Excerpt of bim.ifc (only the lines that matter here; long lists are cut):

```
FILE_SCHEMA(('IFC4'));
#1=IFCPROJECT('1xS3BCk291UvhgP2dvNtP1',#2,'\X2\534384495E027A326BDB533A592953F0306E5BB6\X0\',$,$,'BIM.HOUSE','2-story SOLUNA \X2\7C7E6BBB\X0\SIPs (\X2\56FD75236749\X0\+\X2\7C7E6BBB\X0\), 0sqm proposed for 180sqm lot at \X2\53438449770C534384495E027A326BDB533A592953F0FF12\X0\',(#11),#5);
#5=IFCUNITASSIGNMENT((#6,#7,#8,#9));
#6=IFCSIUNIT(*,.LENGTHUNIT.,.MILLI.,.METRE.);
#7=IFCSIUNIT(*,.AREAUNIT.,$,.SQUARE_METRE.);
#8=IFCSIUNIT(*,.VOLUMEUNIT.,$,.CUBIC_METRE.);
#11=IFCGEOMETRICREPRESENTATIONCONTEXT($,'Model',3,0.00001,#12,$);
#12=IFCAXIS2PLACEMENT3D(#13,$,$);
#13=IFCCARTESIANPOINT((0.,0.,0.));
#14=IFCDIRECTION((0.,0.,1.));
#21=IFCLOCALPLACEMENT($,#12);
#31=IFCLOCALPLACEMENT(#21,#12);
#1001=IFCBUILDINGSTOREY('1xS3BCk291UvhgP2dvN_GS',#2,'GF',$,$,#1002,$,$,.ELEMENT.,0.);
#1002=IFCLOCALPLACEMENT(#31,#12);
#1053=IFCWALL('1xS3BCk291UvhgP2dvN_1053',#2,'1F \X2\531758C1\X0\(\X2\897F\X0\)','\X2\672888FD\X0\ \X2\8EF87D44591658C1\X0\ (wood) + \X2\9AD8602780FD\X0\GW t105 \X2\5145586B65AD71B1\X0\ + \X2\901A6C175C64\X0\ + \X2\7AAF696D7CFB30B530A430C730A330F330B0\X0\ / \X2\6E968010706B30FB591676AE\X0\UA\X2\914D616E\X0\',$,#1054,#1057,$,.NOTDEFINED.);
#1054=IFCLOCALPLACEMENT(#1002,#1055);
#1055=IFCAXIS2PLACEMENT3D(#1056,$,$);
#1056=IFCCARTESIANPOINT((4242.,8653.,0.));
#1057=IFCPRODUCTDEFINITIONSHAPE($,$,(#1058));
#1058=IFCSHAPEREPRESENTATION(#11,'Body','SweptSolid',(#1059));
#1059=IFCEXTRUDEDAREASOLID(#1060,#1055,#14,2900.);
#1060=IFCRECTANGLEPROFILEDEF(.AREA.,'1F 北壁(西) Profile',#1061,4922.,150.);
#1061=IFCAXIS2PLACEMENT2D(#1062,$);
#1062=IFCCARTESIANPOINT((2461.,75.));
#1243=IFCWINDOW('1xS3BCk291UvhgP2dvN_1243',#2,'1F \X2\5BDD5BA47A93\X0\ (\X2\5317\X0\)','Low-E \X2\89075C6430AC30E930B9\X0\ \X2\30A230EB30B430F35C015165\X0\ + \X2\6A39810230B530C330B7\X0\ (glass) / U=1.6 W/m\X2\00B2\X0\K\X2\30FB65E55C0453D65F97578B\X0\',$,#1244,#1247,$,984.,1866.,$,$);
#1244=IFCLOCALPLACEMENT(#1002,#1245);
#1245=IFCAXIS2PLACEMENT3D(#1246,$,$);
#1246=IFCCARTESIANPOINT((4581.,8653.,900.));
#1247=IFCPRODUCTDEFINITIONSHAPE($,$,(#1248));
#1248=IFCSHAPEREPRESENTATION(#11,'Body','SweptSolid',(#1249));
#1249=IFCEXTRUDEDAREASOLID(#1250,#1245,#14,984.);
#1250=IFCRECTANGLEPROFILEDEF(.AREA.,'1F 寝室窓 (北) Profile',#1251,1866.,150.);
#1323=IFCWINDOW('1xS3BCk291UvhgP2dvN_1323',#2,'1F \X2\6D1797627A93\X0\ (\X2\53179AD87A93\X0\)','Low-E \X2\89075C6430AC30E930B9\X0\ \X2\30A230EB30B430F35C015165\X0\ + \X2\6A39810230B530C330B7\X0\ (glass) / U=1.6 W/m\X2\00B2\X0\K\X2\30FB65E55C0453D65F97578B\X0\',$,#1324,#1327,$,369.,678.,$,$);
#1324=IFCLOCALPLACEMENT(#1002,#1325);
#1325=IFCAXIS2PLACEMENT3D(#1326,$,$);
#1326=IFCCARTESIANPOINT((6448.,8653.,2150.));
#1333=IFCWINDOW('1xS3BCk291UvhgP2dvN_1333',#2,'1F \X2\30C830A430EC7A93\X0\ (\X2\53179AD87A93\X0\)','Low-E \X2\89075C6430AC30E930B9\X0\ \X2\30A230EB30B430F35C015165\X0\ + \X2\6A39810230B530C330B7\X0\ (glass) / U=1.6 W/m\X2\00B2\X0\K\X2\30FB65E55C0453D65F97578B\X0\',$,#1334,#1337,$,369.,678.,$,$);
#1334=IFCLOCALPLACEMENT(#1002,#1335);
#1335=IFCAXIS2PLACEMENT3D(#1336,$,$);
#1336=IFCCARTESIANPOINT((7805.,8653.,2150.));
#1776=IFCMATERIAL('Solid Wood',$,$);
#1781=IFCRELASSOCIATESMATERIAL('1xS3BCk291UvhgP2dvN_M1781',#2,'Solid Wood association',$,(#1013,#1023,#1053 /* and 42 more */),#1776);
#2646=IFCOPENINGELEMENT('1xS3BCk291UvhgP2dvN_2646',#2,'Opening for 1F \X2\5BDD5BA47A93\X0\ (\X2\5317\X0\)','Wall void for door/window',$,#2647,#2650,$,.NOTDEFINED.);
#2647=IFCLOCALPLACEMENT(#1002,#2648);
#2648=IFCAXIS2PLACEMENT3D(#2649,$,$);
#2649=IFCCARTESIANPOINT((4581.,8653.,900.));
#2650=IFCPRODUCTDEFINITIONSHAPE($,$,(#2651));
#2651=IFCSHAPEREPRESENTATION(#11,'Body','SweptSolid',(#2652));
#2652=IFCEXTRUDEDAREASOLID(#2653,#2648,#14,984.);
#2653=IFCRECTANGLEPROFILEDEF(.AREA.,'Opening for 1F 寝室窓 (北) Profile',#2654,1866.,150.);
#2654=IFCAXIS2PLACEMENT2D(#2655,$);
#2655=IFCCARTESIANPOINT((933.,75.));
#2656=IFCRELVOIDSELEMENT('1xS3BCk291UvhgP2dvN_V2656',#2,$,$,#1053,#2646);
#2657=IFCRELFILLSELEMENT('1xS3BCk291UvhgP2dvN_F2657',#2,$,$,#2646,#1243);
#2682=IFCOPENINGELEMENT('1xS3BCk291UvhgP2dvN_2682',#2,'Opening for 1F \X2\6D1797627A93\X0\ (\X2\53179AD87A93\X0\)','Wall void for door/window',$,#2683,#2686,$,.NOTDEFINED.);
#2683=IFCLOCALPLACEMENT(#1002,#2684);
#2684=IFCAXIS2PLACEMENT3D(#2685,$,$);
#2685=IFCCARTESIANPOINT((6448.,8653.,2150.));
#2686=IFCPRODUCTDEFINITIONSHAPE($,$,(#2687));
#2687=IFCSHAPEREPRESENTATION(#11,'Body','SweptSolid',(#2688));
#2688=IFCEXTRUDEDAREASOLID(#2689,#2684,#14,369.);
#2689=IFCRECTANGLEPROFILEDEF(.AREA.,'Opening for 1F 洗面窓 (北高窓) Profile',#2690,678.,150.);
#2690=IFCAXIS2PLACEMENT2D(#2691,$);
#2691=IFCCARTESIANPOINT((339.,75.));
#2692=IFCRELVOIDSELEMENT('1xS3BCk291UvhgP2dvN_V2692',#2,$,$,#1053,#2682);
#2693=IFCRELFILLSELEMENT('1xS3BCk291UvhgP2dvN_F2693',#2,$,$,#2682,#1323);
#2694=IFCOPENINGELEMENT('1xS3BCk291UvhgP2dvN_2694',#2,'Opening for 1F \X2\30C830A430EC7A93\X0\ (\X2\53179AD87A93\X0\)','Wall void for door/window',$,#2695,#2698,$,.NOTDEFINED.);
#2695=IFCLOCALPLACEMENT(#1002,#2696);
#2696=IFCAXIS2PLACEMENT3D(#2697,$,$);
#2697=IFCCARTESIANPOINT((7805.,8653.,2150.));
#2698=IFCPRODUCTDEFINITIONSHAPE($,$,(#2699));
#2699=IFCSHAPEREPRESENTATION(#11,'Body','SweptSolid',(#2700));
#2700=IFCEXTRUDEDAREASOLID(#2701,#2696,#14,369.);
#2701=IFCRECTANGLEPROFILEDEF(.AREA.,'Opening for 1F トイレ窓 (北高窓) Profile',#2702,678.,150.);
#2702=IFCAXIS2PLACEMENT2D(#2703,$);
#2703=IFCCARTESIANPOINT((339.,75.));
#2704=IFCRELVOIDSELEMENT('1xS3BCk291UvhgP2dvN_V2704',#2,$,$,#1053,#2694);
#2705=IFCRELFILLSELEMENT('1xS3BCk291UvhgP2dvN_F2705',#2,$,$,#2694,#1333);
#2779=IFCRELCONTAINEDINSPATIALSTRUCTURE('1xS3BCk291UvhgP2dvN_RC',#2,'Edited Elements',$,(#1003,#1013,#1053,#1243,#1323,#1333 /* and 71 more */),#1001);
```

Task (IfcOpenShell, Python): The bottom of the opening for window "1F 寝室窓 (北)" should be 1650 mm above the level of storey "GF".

```python
import numpy as np
import ifcopenshell
import ifcopenshell.api.geometry
import ifcopenshell.geom
import ifcopenshell.util.element
import ifcopenshell.util.placement
import ifcopenshell.util.shape
import ifcopenshell.util.unit

model = ifcopenshell.open("bim.ifc")
unit_scale = ifcopenshell.util.unit.calculate_unit_scale(model)

window = model.by_guid("1xS3BCk291UvhgP2dvN_1243")
opening = window.FillsVoids[0].RelatingOpeningElement
storey = ifcopenshell.util.element.get_container(window, ifc_class="IfcBuildingStorey")
level = ifcopenshell.util.placement.get_local_placement(storey.ObjectPlacement)[2, 3]

# The opening's origin need not be at the sill, so measure its lowest point.
shape = ifcopenshell.geom.create_shape(ifcopenshell.geom.settings(), opening)
bottom = ifcopenshell.util.shape.get_shape_bottom_elevation(shape, shape.geometry) / unit_scale
dz = level + 1650.0 - bottom

shift = np.array([0.0, 0.0, dz])
# The window is not placed relative to its opening, so move both.
for product in (opening, window):
    matrix = ifcopenshell.util.placement.get_local_placement(product.ObjectPlacement)
    matrix[:3, 3] += shift
    ifcopenshell.api.geometry.edit_object_placement(model, product=product, matrix=matrix, is_si=False)

print(f"moved by {dz * unit_scale:+.3f} m")

model.write("bim_updated.ifc")
```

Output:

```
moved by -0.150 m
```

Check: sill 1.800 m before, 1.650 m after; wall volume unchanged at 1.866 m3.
